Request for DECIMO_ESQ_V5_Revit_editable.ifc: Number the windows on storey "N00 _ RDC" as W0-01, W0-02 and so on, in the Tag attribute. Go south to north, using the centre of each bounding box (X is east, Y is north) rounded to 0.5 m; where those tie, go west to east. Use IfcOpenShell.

First a look at what the model holds.

```python
import ifcopenshell
import ifcopenshell.util.element
import ifcopenshell.util.placement

model = ifcopenshell.open("DECIMO_ESQ_V5_Revit_editable.ifc")
print(model.schema)
storey = next(s for s in model.by_type("IfcBuildingStorey") if s.Name == "N00 _ RDC")
windows = [e for e in ifcopenshell.util.element.get_decomposition(storey) if e.is_a("IfcWindow")]
for e in sorted(windows, key=lambda e: e.id()):
    origin = ifcopenshell.util.placement.get_local_placement(e.ObjectPlacement)[:3, 3]
    print(e.id(), e.Tag, e.Name, origin.round(2) + 0.0, sep=" | ")
```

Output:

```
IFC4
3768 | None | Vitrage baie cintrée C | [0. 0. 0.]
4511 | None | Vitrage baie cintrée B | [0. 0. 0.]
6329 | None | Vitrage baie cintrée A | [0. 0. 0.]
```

```python
import ifcopenshell
import ifcopenshell.geom
import ifcopenshell.util.element
import ifcopenshell.util.shape

model = ifcopenshell.open("DECIMO_ESQ_V5_Revit_editable.ifc")
settings = ifcopenshell.geom.settings()
settings.set("use-world-coords", True)


def centre(element):
    shape = ifcopenshell.geom.create_shape(settings, element)
    return ifcopenshell.util.shape.get_bbox_centroid(shape.geometry)


storey = next(s for s in model.by_type("IfcBuildingStorey") if s.Name == "N00 _ RDC")
windows = [e for e in ifcopenshell.util.element.get_decomposition(storey) if e.is_a("IfcWindow")]

# Insertion points can sit at a corner or the storey origin, so sort by the geometry (in metres).
centres = {e: centre(e) for e in windows}
windows.sort(key=lambda e: (round(centres[e][1] / 0.5), centres[e][0]))

for i, e in enumerate(windows, start=1):
    number = f"W0-{i:02d}"
    e.Tag = number
    print(e.id(), number)

model.write("DECIMO_ESQ_V5_Revit_editable_updated.ifc")
```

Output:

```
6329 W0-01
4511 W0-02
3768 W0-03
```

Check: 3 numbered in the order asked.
